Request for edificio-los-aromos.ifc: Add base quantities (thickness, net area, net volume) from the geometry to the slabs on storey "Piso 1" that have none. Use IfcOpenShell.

First a look at what the model holds.

```python
import ifcopenshell
import ifcopenshell.util.element
import ifcopenshell.util.unit

model = ifcopenshell.open("edificio-los-aromos.ifc")
print(model.schema)
for unit_type in ("LENGTHUNIT", "AREAUNIT", "VOLUMEUNIT"):
    print(unit_type, ifcopenshell.util.unit.calculate_unit_scale(model, unit_type))
storey = next(s for s in model.by_type("IfcBuildingStorey") if s.Name == "Piso 1")
slabs = [e for e in ifcopenshell.util.element.get_decomposition(storey) if e.is_a("IfcSlab")]
for e in sorted(slabs, key=lambda e: e.id()):
    print(e.id(), e.is_a(), e.Name, list(ifcopenshell.util.element.get_psets(e, qtos_only=True)), sep=" | ")
```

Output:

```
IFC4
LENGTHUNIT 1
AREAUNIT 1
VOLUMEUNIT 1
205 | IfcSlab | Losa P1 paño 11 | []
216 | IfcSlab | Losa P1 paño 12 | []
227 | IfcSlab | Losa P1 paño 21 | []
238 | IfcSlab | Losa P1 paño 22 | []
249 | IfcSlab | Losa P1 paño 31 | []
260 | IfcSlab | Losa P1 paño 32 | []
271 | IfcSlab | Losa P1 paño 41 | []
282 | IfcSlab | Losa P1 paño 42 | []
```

```python
import ifcopenshell
import ifcopenshell.api.pset
import ifcopenshell.geom
import ifcopenshell.util.element
import ifcopenshell.util.shape
import ifcopenshell.util.unit

model = ifcopenshell.open("edificio-los-aromos.ifc")
unit_scale = ifcopenshell.util.unit.calculate_unit_scale(model)
area_scale = ifcopenshell.util.unit.calculate_unit_scale(model, "AREAUNIT")
volume_scale = ifcopenshell.util.unit.calculate_unit_scale(model, "VOLUMEUNIT")
settings = ifcopenshell.geom.settings()

storey = next(s for s in model.by_type("IfcBuildingStorey") if s.Name == "Piso 1")
slabs = [e for e in ifcopenshell.util.element.get_decomposition(storey) if e.is_a("IfcSlab")]

for e in sorted(slabs, key=lambda e: e.id()):
    if ifcopenshell.util.element.get_psets(e, qtos_only=True, should_inherit=False):
        continue
    # Geometry comes back in metres, in the element's own axes.
    shape = ifcopenshell.geom.create_shape(settings, e)
    values = {
        "Width": ifcopenshell.util.shape.get_z(shape.geometry) / unit_scale,
        "NetArea": ifcopenshell.util.shape.get_footprint_area(shape.geometry) / area_scale,
        "NetVolume": ifcopenshell.util.shape.get_volume(shape.geometry) / volume_scale,
    }
    qto = ifcopenshell.api.pset.add_qto(model, product=e, name="Qto_SlabBaseQuantities")
    ifcopenshell.api.pset.edit_qto(model, qto=qto, properties=values)
    print(e.id(), {k: round(v, 3) for k, v in values.items()})

model.write("edificio-los-aromos_edited.ifc")
```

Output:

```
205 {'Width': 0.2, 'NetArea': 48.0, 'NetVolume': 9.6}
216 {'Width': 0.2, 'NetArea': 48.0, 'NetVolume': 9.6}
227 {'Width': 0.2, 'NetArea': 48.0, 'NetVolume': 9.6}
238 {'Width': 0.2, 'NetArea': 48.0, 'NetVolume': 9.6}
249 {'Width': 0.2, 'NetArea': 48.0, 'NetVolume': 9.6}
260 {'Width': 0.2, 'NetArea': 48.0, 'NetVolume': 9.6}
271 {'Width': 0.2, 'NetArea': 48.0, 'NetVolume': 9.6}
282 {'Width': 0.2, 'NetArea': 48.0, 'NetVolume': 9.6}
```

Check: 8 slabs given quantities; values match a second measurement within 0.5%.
